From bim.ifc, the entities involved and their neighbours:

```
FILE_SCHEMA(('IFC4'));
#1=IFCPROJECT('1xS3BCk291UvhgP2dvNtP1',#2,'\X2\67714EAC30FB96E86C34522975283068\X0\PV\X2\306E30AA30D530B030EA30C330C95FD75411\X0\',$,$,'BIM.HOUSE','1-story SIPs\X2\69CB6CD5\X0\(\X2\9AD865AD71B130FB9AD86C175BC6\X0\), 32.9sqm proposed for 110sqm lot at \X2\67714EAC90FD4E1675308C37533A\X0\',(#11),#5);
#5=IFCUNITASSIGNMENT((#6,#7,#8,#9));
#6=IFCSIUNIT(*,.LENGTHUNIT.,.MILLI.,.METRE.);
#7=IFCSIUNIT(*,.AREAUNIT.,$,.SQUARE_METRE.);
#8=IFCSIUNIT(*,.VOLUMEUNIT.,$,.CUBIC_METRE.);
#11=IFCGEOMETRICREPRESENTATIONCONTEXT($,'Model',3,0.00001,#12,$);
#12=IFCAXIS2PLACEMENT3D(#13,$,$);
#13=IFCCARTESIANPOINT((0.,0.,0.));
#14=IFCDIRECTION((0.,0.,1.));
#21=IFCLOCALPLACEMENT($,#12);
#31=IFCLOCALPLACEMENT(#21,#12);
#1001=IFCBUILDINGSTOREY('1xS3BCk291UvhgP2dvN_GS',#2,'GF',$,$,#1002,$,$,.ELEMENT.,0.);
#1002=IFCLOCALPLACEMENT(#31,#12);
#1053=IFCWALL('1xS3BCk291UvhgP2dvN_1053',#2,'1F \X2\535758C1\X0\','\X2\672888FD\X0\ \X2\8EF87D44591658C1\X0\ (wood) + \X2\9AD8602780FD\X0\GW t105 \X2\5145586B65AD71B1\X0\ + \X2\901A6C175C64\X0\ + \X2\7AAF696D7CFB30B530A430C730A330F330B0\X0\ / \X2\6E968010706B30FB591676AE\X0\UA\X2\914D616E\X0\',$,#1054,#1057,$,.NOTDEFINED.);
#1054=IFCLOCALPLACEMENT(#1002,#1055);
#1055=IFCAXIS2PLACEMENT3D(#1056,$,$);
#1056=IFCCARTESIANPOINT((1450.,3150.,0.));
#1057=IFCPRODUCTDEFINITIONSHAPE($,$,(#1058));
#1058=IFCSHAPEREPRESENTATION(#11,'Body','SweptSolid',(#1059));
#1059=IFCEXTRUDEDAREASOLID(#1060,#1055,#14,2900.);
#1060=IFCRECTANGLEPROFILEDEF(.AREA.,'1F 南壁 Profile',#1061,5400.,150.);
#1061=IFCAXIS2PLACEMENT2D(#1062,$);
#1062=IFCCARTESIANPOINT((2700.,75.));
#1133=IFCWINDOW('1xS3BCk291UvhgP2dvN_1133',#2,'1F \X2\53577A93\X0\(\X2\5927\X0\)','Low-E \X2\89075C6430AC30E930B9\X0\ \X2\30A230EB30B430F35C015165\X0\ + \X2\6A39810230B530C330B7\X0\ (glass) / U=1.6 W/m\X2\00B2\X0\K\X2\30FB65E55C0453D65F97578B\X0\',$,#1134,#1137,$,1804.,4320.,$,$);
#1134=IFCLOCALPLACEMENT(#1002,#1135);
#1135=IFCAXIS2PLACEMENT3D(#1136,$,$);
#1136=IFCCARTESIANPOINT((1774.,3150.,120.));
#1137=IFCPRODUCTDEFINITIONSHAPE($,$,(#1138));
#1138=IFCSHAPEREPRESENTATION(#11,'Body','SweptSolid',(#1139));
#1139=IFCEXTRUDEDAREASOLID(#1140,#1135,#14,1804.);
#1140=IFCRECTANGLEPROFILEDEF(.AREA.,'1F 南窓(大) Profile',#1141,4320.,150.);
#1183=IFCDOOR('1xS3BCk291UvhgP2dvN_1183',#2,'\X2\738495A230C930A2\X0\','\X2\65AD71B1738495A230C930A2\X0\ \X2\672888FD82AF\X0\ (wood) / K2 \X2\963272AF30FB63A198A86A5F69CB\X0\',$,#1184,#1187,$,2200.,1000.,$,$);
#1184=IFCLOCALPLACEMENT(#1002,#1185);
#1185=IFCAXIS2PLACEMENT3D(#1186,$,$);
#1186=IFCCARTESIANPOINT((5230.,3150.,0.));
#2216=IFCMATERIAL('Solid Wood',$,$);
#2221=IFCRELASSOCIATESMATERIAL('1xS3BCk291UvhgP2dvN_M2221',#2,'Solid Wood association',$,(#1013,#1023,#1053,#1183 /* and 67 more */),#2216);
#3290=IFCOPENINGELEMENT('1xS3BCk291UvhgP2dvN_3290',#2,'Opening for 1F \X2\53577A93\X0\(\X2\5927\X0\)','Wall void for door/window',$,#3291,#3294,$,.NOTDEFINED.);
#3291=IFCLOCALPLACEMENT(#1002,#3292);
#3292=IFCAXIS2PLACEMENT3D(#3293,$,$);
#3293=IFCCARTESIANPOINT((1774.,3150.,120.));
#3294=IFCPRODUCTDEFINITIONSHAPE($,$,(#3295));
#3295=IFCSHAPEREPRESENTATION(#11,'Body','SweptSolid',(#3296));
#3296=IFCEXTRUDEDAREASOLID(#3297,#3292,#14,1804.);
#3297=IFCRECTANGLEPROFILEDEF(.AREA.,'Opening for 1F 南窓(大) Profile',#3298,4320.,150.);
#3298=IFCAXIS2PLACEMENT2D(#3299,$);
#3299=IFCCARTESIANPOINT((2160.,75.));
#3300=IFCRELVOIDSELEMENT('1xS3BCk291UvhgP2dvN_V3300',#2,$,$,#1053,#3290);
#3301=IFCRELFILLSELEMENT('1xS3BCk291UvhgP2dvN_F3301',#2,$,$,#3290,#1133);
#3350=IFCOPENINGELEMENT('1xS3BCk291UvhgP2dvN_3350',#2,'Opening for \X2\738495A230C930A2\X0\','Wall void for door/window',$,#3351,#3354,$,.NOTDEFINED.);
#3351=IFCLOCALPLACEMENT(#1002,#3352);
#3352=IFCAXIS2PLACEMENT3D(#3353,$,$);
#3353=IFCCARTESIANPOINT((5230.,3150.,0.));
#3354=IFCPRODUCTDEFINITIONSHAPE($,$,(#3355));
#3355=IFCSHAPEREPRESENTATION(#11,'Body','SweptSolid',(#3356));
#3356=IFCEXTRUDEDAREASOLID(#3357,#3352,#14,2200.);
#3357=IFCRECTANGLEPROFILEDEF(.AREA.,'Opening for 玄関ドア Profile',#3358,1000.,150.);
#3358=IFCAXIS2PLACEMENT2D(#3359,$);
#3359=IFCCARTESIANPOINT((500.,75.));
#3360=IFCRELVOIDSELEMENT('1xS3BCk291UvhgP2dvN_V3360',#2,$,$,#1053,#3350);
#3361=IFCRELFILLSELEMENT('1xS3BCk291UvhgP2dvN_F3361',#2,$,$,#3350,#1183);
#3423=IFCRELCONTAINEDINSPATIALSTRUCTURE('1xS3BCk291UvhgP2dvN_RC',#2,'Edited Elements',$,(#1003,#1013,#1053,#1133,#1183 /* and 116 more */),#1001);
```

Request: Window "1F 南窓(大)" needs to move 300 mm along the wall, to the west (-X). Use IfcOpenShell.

```python
import ifcopenshell
import ifcopenshell.api.geometry
import ifcopenshell.util.placement

model = ifcopenshell.open("bim.ifc")

window = model.by_guid("1xS3BCk291UvhgP2dvN_1133")
opening = window.FillsVoids[0].RelatingOpeningElement
wall = opening.VoidsElements[0].RelatingBuildingElement

wall_matrix = ifcopenshell.util.placement.get_local_placement(wall.ObjectPlacement)
shift = wall_matrix[:3, 0] * -300.0
before = ifcopenshell.util.placement.get_local_placement(window.ObjectPlacement)[:3, 3].copy()

# The window is not placed relative to its opening, so move both.
for product in (opening, window):
    matrix = ifcopenshell.util.placement.get_local_placement(product.ObjectPlacement)
    matrix[:3, 3] += shift
    ifcopenshell.api.geometry.edit_object_placement(model, product=product, matrix=matrix, is_si=False)

after = ifcopenshell.util.placement.get_local_placement(window.ObjectPlacement)[:3, 3]
print("window moved by", (after - before).round(3) + 0.0)

model.write("bim_rev.ifc")
```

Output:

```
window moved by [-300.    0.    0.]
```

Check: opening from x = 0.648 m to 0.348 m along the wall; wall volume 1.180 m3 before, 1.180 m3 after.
